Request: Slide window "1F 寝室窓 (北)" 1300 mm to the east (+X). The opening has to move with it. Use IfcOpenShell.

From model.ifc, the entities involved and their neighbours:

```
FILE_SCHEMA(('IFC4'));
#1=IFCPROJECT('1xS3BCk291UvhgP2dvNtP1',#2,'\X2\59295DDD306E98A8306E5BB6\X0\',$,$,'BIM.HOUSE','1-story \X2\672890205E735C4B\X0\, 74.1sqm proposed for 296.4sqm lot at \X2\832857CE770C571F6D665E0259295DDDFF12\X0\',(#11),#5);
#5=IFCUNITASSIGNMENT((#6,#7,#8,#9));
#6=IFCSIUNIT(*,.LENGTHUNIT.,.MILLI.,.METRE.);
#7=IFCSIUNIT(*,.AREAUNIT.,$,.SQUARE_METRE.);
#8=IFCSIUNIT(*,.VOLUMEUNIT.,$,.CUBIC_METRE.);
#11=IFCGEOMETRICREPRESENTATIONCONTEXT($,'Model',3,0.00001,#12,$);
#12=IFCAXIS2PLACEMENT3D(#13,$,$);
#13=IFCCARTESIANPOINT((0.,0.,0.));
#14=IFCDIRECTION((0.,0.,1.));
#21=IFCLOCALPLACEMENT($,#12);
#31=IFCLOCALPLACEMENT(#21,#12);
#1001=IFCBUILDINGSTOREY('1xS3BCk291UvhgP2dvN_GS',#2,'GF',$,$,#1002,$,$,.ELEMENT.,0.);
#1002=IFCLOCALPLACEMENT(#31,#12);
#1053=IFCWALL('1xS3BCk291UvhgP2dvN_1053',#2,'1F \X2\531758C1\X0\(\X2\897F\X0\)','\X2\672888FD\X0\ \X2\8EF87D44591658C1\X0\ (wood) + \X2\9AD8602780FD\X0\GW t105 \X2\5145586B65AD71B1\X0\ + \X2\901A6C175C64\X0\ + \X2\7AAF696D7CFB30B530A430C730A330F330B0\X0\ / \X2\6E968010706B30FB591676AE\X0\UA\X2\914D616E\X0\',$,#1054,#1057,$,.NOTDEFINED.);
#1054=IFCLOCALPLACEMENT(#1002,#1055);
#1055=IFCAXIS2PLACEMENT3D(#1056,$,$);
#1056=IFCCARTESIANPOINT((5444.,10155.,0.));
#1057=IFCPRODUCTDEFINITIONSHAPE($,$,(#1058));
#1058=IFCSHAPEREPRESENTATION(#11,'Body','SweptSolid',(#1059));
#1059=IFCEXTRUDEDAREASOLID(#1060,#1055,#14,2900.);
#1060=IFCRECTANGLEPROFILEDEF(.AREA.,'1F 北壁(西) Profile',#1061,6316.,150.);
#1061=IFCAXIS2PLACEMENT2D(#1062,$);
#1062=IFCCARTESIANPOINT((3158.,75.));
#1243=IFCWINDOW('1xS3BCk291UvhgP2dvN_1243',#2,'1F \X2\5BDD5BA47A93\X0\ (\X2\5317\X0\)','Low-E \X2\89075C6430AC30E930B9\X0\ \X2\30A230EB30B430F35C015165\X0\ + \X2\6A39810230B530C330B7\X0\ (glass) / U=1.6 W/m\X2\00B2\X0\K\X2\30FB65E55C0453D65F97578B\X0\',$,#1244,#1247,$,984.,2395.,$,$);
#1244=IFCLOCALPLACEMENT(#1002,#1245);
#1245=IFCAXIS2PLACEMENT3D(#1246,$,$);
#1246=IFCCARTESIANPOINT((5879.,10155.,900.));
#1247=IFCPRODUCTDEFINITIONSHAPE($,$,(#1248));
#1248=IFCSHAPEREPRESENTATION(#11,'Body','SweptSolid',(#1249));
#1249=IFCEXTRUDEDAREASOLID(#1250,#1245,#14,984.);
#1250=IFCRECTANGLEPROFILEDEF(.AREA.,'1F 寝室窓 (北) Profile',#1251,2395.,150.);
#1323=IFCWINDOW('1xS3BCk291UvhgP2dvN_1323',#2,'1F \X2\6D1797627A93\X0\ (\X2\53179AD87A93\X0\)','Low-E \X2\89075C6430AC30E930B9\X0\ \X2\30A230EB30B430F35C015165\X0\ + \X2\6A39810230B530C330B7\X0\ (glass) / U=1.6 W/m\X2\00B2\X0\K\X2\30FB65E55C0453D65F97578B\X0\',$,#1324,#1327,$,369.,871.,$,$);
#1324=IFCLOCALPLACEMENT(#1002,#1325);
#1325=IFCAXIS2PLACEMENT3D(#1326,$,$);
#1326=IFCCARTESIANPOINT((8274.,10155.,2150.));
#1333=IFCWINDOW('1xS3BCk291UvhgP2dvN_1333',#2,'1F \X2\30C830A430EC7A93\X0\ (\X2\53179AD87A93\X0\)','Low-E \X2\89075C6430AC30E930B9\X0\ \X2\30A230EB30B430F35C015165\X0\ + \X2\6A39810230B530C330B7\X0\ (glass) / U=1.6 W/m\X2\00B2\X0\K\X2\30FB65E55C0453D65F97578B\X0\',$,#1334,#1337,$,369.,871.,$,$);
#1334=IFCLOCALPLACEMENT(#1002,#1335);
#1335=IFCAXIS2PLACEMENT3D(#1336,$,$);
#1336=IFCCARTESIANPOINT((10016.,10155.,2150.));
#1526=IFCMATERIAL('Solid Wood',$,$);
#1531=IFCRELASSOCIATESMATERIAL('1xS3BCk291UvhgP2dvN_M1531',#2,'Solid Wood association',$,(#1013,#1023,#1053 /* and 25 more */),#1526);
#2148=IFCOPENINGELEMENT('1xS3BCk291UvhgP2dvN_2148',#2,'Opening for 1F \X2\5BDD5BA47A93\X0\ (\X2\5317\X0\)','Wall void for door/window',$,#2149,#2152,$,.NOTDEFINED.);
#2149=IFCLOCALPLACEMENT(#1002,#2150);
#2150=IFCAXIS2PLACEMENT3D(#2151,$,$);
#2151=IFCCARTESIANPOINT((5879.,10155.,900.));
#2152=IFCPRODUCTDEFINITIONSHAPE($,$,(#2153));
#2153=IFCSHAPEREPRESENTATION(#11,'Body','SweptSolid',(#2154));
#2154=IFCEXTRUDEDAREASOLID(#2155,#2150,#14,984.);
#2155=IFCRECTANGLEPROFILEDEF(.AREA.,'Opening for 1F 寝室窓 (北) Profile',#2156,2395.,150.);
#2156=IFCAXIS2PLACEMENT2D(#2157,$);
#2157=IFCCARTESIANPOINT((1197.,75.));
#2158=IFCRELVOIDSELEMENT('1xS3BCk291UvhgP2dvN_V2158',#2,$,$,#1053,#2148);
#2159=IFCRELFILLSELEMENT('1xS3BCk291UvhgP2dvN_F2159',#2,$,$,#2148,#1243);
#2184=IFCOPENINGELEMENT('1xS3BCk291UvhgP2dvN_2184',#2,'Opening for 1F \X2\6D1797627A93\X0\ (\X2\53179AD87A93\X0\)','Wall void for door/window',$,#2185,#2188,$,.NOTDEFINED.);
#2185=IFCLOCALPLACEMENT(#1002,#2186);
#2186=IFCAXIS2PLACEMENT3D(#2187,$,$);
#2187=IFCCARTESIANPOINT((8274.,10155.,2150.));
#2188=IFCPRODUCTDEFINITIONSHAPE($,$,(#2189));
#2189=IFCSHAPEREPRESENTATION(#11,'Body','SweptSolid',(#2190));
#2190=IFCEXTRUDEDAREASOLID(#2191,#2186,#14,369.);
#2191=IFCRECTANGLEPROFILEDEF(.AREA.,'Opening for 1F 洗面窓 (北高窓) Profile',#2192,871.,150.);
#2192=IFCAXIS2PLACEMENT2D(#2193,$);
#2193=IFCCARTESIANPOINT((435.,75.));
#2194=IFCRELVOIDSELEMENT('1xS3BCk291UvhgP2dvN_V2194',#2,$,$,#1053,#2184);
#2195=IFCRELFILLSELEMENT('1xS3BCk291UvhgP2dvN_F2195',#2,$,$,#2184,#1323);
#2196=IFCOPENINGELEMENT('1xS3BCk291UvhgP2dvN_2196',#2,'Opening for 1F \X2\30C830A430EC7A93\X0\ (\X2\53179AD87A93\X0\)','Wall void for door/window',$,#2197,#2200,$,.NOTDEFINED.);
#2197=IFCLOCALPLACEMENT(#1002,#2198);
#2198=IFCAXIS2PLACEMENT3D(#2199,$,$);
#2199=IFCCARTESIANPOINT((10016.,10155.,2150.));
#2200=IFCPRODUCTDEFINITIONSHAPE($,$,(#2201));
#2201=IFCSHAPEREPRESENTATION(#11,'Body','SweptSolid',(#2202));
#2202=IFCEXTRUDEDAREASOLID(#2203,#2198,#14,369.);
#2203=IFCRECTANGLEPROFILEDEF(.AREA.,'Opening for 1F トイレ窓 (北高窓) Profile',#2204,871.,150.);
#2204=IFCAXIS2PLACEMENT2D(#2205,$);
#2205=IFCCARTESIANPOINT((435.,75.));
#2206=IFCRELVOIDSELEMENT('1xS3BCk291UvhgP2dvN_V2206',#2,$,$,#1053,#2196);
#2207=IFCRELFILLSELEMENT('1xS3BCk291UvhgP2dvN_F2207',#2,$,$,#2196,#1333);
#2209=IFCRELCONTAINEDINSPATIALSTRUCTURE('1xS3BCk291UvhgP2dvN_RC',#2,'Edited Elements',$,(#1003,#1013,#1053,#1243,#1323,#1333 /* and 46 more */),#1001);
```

```python
import ifcopenshell
import ifcopenshell.api.geometry
import ifcopenshell.util.placement
import ifcopenshell.util.unit

model = ifcopenshell.open("model.ifc")
unit_scale = ifcopenshell.util.unit.calculate_unit_scale(model)

window = model.by_guid("1xS3BCk291UvhgP2dvN_1243")
opening = window.FillsVoids[0].RelatingOpeningElement
wall = opening.VoidsElements[0].RelatingBuildingElement

wall_matrix = ifcopenshell.util.placement.get_local_placement(wall.ObjectPlacement)
shift = wall_matrix[:3, 0] * 1.3 / unit_scale
before = ifcopenshell.util.placement.get_local_placement(window.ObjectPlacement)[:3, 3].copy()

# The window is not placed relative to its opening, so move both.
for product in (opening, window):
    matrix = ifcopenshell.util.placement.get_local_placement(product.ObjectPlacement)
    matrix[:3, 3] += shift
    ifcopenshell.api.geometry.edit_object_placement(model, product=product, matrix=matrix, is_si=False)

after = ifcopenshell.util.placement.get_local_placement(window.ObjectPlacement)[:3, 3]
print("window moved by", (after - before).round(3) + 0.0)

model.write("model_edited.ifc")
```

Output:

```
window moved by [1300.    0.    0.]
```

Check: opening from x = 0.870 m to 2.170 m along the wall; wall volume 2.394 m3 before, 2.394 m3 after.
